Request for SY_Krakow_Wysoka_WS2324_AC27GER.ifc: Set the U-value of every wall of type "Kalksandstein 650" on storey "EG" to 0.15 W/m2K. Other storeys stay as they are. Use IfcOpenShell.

First a look at what the model holds.

```python
import ifcopenshell
import ifcopenshell.util.element

model = ifcopenshell.open("SY_Krakow_Wysoka_WS2324_AC27GER.ifc")
print(model.schema)
storey = next(s for s in model.by_type("IfcBuildingStorey") if s.Name == "EG")
walls = [e for e in ifcopenshell.util.element.get_decomposition(storey) if e.is_a("IfcWall")]
seen = {}
for e in walls:
    element_type = ifcopenshell.util.element.get_type(e)
    key = (element_type.Name if element_type != e and element_type else None, ifcopenshell.util.element.get_pset(e, "Pset_WallCommon", "ThermalTransmittance"))
    seen[key] = seen.get(key, 0) + 1
for (name, value), count in sorted(seen.items(), key=str):
    print(count, "x", name, "|", value)
```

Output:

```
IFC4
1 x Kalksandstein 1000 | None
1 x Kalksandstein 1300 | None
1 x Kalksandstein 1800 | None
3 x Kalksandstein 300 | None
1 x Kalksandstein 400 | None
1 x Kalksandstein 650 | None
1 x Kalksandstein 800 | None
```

```python
import ifcopenshell
import ifcopenshell.api.pset
import ifcopenshell.util.element

model = ifcopenshell.open("SY_Krakow_Wysoka_WS2324_AC27GER.ifc")

storey = next(s for s in model.by_type("IfcBuildingStorey") if s.Name == "EG")
walls = [e for e in ifcopenshell.util.element.get_decomposition(storey) if e.is_a("IfcWall")]

count = 0
for e in walls:
    element_type = ifcopenshell.util.element.get_type(e)
    if element_type in (None, e) or element_type.Name != "Kalksandstein 650":
        continue
    # add_pset returns the element's existing set when there is one.
    pset = ifcopenshell.api.pset.add_pset(model, product=e, name="Pset_WallCommon")
    ifcopenshell.api.pset.edit_pset(model, pset=pset, properties={"ThermalTransmittance": 0.15})
    count += 1

print(count, "walls updated")

model.write("SY_Krakow_Wysoka_WS2324_AC27GER_v2.ifc")
```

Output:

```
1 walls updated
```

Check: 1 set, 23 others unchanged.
